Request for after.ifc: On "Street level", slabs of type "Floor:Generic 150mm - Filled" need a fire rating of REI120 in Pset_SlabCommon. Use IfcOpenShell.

First a look at what the model holds.

```python
import ifcopenshell
import ifcopenshell.util.element

model = ifcopenshell.open("after.ifc")
print(model.schema)
storey = next(s for s in model.by_type("IfcBuildingStorey") if s.Name == "Street level")
slabs = [e for e in ifcopenshell.util.element.get_decomposition(storey) if e.is_a("IfcSlab")]
seen = {}
for e in slabs:
    element_type = ifcopenshell.util.element.get_type(e)
    key = (element_type.Name if element_type != e and element_type else None, ifcopenshell.util.element.get_pset(e, "Pset_SlabCommon", "FireRating"))
    seen[key] = seen.get(key, 0) + 1
for (name, value), count in sorted(seen.items(), key=str):
    print(count, "x", name, "|", value)
```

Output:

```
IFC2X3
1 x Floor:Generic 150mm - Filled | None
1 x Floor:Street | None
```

```python
import ifcopenshell
import ifcopenshell.api.pset
import ifcopenshell.util.element

model = ifcopenshell.open("after.ifc")

storey = next(s for s in model.by_type("IfcBuildingStorey") if s.Name == "Street level")
slabs = [e for e in ifcopenshell.util.element.get_decomposition(storey) if e.is_a("IfcSlab")]

count = 0
for e in slabs:
    element_type = ifcopenshell.util.element.get_type(e)
    if element_type in (None, e) or element_type.Name != "Floor:Generic 150mm - Filled":
        continue
    # add_pset returns the element's existing set when there is one.
    pset = ifcopenshell.api.pset.add_pset(model, product=e, name="Pset_SlabCommon")
    ifcopenshell.api.pset.edit_pset(model, pset=pset, properties={"FireRating": "REI120"})
    count += 1

print(count, "slabs updated")

model.write("after_rev.ifc")
```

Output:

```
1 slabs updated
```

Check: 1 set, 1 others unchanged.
